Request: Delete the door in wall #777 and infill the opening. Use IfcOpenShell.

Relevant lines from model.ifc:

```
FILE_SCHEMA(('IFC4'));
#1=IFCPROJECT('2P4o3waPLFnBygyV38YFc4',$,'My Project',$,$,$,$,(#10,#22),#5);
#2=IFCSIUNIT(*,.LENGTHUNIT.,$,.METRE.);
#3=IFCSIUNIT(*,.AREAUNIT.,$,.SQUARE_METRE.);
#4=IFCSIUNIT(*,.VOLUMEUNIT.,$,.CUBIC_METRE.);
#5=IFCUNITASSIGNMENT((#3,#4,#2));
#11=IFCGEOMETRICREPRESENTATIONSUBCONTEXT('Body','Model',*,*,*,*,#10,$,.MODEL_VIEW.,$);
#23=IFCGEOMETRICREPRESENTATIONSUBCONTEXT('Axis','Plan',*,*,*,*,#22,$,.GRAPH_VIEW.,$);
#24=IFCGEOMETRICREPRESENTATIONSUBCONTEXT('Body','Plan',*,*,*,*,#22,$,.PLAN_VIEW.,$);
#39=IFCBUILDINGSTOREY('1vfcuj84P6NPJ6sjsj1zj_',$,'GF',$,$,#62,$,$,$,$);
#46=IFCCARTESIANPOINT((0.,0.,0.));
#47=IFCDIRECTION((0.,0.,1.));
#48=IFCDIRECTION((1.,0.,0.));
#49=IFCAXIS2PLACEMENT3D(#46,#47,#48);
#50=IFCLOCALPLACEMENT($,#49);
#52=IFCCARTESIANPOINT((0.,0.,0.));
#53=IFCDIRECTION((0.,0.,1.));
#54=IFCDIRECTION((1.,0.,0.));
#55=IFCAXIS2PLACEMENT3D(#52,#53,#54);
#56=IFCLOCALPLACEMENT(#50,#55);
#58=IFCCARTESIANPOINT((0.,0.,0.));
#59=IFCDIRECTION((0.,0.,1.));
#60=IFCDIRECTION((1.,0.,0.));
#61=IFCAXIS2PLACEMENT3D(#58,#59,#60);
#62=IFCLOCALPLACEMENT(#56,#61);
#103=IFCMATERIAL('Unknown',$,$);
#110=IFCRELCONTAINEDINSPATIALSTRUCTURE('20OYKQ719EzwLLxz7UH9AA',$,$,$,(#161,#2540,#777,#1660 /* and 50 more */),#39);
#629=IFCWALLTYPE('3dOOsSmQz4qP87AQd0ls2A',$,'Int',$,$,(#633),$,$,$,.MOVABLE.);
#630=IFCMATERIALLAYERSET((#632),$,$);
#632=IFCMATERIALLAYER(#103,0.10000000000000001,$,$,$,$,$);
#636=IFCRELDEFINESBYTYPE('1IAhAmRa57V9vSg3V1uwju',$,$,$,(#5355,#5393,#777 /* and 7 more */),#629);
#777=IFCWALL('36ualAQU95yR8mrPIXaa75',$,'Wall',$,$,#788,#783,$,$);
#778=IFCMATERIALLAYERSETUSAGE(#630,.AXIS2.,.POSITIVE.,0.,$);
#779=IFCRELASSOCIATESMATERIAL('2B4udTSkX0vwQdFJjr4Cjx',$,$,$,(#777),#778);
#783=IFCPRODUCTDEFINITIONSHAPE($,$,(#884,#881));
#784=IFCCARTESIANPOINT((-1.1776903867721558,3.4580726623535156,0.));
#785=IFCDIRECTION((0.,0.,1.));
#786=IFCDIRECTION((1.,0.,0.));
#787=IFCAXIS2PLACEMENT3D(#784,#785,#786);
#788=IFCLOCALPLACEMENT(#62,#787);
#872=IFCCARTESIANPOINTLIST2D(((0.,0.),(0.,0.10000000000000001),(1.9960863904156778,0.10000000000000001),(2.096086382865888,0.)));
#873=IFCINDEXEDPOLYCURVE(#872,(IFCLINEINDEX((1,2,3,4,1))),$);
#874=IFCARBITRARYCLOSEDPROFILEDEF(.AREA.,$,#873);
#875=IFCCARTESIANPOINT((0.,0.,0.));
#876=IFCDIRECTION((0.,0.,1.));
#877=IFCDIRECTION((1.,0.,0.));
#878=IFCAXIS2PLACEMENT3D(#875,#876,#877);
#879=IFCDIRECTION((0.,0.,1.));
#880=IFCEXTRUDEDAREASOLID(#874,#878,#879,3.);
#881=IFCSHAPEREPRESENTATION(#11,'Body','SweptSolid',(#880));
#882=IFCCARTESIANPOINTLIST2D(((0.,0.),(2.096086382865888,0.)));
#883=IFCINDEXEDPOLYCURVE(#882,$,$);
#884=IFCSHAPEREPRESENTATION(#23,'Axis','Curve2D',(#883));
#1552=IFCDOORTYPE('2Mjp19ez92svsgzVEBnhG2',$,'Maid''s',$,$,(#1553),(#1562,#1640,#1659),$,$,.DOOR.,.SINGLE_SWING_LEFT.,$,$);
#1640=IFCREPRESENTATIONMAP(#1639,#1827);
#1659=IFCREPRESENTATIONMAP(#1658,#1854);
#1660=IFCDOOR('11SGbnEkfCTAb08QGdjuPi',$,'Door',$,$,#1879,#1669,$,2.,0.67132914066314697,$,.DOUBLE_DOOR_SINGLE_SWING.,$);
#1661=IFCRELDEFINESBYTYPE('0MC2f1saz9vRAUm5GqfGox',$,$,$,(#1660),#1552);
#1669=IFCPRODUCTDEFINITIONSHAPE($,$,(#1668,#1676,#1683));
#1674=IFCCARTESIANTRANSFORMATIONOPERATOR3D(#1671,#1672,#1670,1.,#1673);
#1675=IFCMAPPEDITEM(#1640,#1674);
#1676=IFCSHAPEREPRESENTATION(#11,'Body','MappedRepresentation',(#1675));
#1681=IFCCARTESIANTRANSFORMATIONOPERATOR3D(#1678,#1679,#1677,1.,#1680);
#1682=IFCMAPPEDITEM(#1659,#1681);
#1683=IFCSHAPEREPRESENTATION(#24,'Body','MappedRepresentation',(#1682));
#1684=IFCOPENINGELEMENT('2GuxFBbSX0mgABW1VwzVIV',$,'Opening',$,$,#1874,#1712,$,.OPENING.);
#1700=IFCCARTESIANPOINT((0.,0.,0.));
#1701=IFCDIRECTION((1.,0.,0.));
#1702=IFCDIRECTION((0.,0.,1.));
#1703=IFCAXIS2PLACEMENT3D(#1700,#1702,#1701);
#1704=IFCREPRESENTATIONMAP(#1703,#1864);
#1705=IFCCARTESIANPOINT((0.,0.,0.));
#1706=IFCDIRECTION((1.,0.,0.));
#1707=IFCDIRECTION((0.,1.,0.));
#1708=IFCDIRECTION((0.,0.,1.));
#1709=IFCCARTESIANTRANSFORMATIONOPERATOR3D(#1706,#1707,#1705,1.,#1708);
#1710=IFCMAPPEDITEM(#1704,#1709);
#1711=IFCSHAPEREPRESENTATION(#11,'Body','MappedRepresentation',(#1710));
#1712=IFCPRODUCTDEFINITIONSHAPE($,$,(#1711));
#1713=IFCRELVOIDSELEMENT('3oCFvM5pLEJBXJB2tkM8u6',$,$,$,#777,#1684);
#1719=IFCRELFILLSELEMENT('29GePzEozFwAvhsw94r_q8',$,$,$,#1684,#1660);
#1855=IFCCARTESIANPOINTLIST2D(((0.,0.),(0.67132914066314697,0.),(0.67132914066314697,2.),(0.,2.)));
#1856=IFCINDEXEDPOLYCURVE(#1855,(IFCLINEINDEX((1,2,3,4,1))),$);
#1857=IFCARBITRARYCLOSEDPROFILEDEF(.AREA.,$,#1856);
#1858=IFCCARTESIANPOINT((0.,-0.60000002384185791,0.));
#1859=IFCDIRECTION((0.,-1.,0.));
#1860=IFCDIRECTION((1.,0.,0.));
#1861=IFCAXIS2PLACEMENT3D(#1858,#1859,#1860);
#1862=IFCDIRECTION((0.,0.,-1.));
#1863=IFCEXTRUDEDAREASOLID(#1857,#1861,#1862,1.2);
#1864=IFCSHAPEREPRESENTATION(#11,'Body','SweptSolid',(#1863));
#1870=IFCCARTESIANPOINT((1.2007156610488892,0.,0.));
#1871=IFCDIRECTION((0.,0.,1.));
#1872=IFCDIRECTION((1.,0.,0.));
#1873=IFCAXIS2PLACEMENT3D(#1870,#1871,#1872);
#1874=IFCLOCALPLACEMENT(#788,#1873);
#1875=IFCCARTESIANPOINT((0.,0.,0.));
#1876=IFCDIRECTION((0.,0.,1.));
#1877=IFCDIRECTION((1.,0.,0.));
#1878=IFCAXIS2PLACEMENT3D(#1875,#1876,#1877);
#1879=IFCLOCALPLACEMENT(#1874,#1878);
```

```python
import ifcopenshell
import ifcopenshell.api.feature
import ifcopenshell.api.root
import ifcopenshell.geom
import ifcopenshell.util.shape

model = ifcopenshell.open("model.ifc")
settings = ifcopenshell.geom.settings()


def volume(element):
    """Net volume in cubic metres, openings subtracted."""
    shape = ifcopenshell.geom.create_shape(settings, element)
    return ifcopenshell.util.shape.get_volume(shape.geometry)


door = model.by_guid("11SGbnEkfCTAb08QGdjuPi")
opening = door.FillsVoids[0].RelatingOpeningElement
wall = opening.VoidsElements[0].RelatingBuildingElement
before = volume(wall)

ifcopenshell.api.root.remove_product(model, product=door)
ifcopenshell.api.feature.remove_feature(model, feature=opening)

after = volume(wall)

print(f"wall volume {before:.3f} -> {after:.3f} m3")

model.write("model_v2.ifc")
```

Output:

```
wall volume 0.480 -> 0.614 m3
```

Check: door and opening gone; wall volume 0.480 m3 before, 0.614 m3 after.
